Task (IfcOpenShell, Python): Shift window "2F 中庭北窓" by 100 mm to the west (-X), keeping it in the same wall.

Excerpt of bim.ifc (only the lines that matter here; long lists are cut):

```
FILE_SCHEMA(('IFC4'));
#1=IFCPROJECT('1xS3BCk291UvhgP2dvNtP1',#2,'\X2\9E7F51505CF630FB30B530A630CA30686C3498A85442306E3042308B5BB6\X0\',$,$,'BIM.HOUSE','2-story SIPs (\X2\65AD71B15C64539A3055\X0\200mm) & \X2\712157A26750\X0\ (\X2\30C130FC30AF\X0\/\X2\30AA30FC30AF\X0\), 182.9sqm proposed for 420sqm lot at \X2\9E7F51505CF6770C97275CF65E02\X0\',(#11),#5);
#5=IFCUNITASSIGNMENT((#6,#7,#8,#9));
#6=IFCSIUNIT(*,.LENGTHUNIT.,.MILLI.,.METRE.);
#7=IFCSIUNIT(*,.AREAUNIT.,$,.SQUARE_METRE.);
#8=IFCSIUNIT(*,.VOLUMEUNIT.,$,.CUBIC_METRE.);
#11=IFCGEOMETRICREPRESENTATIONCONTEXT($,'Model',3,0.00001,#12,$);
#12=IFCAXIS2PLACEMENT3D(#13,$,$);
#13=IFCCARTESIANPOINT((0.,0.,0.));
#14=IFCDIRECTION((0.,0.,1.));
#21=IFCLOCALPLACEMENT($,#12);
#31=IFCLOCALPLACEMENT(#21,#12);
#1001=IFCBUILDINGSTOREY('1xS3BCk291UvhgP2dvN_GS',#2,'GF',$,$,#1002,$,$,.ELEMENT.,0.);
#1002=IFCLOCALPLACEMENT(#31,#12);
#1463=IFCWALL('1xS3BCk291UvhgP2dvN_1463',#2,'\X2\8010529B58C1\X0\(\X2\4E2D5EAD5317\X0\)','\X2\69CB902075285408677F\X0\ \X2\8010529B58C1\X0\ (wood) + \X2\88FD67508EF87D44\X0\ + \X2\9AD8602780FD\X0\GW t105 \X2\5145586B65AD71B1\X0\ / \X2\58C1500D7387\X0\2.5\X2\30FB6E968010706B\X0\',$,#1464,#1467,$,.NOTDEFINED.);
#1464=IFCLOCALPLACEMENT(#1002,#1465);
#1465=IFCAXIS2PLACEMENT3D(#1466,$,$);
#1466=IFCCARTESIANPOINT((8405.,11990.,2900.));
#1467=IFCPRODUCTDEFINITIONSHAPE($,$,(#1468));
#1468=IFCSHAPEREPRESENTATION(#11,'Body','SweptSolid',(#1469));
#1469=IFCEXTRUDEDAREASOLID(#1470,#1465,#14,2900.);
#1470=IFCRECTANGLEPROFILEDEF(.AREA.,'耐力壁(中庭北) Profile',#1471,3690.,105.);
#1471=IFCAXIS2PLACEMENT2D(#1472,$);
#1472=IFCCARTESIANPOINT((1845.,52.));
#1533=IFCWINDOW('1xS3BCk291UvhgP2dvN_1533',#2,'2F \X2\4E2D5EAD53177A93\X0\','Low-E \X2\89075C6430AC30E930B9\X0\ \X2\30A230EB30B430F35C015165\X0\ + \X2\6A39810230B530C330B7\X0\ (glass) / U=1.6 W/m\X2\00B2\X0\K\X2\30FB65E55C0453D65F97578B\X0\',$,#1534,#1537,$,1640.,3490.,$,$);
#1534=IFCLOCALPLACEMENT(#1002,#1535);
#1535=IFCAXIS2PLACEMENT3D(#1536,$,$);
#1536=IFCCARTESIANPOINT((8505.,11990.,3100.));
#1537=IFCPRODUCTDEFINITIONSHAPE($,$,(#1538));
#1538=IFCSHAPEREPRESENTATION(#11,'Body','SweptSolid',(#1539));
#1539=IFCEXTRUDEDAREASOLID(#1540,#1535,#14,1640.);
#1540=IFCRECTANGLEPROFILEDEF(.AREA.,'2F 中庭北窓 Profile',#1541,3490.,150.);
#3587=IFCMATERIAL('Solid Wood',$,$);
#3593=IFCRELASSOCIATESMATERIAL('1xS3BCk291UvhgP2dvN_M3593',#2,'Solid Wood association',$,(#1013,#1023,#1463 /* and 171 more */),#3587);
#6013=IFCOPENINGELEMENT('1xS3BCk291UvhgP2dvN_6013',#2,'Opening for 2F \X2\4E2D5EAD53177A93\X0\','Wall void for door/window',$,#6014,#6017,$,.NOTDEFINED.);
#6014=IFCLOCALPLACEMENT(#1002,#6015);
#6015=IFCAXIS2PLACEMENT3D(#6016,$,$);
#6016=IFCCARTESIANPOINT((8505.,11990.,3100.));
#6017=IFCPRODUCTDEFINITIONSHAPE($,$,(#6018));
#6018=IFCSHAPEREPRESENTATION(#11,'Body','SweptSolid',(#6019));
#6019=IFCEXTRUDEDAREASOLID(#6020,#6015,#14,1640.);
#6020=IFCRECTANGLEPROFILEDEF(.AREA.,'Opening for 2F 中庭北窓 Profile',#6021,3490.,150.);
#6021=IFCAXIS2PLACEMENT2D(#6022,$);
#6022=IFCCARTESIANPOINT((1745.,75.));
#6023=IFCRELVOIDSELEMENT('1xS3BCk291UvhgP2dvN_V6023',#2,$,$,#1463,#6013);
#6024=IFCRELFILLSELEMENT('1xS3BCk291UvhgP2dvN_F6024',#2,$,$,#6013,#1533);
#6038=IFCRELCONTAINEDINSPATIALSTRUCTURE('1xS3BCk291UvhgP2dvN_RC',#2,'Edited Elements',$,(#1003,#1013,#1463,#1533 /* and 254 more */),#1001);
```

```python
import ifcopenshell
import ifcopenshell.api.geometry
import ifcopenshell.util.placement
import ifcopenshell.util.unit

model = ifcopenshell.open("bim.ifc")
unit_scale = ifcopenshell.util.unit.calculate_unit_scale(model)

window = model.by_guid("1xS3BCk291UvhgP2dvN_1533")
opening = window.FillsVoids[0].RelatingOpeningElement
wall = opening.VoidsElements[0].RelatingBuildingElement

wall_matrix = ifcopenshell.util.placement.get_local_placement(wall.ObjectPlacement)
shift = wall_matrix[:3, 0] * -0.1 / unit_scale
before = ifcopenshell.util.placement.get_local_placement(window.ObjectPlacement)[:3, 3].copy()

# The window is not placed relative to its opening, so move both.
for product in (opening, window):
    matrix = ifcopenshell.util.placement.get_local_placement(product.ObjectPlacement)
    matrix[:3, 3] += shift
    ifcopenshell.api.geometry.edit_object_placement(model, product=product, matrix=matrix, is_si=False)

after = ifcopenshell.util.placement.get_local_placement(window.ObjectPlacement)[:3, 3]
print("window moved by", (after - before).round(3) + 0.0)

model.write("bim-out.ifc")
```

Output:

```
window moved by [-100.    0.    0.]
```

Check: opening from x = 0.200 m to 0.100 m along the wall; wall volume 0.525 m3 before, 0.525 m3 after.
